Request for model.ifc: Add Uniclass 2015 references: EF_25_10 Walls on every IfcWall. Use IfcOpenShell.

First a look at what the model holds.

```python
import ifcopenshell

model = ifcopenshell.open("model.ifc")
print(model.schema)
print("classifications:", [c.Name for c in model.by_type("IfcClassification")])
for ifc_class in ("IfcDoor", "IfcRoof", "IfcStair", "IfcWall", "IfcWindow"):
    print(ifc_class, len(model.by_type(ifc_class)))
```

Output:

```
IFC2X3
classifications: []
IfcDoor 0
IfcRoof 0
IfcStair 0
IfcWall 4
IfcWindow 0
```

```python
import ifcopenshell
import ifcopenshell.api.classification

model = ifcopenshell.open("model.ifc")

# IFC2X3 requires Source and Edition and has no link from the project to the system.
system = model.create_entity("IfcClassification", Source="NBS", Edition="2015", Name="Uniclass 2015")

codes = {
    "IfcWall": ("EF_25_10", "Walls"),
}
for ifc_class, (code, name) in codes.items():
    products = model.by_type(ifc_class)
    ifcopenshell.api.classification.add_reference(
        model, products=products, classification=system, identification=code, name=name
    )
    print(code, len(products))

model.write("model-out.ifc")
```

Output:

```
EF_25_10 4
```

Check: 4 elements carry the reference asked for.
